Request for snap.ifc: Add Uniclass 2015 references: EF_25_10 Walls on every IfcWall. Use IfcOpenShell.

First a look at what the model holds.

```python
import ifcopenshell

model = ifcopenshell.open("snap.ifc")
print(model.schema)
print("classifications:", [c.Name for c in model.by_type("IfcClassification")])
for ifc_class in ("IfcDoor", "IfcRoof", "IfcStair", "IfcWall", "IfcWindow"):
    print(ifc_class, len(model.by_type(ifc_class)))
```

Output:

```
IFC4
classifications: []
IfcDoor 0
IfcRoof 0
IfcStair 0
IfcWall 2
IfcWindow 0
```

```python
import ifcopenshell
import ifcopenshell.api.classification

model = ifcopenshell.open("snap.ifc")

system = ifcopenshell.api.classification.add_classification(model, classification="Uniclass 2015")

codes = {
    "IfcWall": ("EF_25_10", "Walls"),
}
for ifc_class, (code, name) in codes.items():
    products = model.by_type(ifc_class)
    ifcopenshell.api.classification.add_reference(
        model, products=products, classification=system, identification=code, name=name
    )
    print(code, len(products))

model.write("snap_rev.ifc")
```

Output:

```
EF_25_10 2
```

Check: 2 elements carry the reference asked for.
